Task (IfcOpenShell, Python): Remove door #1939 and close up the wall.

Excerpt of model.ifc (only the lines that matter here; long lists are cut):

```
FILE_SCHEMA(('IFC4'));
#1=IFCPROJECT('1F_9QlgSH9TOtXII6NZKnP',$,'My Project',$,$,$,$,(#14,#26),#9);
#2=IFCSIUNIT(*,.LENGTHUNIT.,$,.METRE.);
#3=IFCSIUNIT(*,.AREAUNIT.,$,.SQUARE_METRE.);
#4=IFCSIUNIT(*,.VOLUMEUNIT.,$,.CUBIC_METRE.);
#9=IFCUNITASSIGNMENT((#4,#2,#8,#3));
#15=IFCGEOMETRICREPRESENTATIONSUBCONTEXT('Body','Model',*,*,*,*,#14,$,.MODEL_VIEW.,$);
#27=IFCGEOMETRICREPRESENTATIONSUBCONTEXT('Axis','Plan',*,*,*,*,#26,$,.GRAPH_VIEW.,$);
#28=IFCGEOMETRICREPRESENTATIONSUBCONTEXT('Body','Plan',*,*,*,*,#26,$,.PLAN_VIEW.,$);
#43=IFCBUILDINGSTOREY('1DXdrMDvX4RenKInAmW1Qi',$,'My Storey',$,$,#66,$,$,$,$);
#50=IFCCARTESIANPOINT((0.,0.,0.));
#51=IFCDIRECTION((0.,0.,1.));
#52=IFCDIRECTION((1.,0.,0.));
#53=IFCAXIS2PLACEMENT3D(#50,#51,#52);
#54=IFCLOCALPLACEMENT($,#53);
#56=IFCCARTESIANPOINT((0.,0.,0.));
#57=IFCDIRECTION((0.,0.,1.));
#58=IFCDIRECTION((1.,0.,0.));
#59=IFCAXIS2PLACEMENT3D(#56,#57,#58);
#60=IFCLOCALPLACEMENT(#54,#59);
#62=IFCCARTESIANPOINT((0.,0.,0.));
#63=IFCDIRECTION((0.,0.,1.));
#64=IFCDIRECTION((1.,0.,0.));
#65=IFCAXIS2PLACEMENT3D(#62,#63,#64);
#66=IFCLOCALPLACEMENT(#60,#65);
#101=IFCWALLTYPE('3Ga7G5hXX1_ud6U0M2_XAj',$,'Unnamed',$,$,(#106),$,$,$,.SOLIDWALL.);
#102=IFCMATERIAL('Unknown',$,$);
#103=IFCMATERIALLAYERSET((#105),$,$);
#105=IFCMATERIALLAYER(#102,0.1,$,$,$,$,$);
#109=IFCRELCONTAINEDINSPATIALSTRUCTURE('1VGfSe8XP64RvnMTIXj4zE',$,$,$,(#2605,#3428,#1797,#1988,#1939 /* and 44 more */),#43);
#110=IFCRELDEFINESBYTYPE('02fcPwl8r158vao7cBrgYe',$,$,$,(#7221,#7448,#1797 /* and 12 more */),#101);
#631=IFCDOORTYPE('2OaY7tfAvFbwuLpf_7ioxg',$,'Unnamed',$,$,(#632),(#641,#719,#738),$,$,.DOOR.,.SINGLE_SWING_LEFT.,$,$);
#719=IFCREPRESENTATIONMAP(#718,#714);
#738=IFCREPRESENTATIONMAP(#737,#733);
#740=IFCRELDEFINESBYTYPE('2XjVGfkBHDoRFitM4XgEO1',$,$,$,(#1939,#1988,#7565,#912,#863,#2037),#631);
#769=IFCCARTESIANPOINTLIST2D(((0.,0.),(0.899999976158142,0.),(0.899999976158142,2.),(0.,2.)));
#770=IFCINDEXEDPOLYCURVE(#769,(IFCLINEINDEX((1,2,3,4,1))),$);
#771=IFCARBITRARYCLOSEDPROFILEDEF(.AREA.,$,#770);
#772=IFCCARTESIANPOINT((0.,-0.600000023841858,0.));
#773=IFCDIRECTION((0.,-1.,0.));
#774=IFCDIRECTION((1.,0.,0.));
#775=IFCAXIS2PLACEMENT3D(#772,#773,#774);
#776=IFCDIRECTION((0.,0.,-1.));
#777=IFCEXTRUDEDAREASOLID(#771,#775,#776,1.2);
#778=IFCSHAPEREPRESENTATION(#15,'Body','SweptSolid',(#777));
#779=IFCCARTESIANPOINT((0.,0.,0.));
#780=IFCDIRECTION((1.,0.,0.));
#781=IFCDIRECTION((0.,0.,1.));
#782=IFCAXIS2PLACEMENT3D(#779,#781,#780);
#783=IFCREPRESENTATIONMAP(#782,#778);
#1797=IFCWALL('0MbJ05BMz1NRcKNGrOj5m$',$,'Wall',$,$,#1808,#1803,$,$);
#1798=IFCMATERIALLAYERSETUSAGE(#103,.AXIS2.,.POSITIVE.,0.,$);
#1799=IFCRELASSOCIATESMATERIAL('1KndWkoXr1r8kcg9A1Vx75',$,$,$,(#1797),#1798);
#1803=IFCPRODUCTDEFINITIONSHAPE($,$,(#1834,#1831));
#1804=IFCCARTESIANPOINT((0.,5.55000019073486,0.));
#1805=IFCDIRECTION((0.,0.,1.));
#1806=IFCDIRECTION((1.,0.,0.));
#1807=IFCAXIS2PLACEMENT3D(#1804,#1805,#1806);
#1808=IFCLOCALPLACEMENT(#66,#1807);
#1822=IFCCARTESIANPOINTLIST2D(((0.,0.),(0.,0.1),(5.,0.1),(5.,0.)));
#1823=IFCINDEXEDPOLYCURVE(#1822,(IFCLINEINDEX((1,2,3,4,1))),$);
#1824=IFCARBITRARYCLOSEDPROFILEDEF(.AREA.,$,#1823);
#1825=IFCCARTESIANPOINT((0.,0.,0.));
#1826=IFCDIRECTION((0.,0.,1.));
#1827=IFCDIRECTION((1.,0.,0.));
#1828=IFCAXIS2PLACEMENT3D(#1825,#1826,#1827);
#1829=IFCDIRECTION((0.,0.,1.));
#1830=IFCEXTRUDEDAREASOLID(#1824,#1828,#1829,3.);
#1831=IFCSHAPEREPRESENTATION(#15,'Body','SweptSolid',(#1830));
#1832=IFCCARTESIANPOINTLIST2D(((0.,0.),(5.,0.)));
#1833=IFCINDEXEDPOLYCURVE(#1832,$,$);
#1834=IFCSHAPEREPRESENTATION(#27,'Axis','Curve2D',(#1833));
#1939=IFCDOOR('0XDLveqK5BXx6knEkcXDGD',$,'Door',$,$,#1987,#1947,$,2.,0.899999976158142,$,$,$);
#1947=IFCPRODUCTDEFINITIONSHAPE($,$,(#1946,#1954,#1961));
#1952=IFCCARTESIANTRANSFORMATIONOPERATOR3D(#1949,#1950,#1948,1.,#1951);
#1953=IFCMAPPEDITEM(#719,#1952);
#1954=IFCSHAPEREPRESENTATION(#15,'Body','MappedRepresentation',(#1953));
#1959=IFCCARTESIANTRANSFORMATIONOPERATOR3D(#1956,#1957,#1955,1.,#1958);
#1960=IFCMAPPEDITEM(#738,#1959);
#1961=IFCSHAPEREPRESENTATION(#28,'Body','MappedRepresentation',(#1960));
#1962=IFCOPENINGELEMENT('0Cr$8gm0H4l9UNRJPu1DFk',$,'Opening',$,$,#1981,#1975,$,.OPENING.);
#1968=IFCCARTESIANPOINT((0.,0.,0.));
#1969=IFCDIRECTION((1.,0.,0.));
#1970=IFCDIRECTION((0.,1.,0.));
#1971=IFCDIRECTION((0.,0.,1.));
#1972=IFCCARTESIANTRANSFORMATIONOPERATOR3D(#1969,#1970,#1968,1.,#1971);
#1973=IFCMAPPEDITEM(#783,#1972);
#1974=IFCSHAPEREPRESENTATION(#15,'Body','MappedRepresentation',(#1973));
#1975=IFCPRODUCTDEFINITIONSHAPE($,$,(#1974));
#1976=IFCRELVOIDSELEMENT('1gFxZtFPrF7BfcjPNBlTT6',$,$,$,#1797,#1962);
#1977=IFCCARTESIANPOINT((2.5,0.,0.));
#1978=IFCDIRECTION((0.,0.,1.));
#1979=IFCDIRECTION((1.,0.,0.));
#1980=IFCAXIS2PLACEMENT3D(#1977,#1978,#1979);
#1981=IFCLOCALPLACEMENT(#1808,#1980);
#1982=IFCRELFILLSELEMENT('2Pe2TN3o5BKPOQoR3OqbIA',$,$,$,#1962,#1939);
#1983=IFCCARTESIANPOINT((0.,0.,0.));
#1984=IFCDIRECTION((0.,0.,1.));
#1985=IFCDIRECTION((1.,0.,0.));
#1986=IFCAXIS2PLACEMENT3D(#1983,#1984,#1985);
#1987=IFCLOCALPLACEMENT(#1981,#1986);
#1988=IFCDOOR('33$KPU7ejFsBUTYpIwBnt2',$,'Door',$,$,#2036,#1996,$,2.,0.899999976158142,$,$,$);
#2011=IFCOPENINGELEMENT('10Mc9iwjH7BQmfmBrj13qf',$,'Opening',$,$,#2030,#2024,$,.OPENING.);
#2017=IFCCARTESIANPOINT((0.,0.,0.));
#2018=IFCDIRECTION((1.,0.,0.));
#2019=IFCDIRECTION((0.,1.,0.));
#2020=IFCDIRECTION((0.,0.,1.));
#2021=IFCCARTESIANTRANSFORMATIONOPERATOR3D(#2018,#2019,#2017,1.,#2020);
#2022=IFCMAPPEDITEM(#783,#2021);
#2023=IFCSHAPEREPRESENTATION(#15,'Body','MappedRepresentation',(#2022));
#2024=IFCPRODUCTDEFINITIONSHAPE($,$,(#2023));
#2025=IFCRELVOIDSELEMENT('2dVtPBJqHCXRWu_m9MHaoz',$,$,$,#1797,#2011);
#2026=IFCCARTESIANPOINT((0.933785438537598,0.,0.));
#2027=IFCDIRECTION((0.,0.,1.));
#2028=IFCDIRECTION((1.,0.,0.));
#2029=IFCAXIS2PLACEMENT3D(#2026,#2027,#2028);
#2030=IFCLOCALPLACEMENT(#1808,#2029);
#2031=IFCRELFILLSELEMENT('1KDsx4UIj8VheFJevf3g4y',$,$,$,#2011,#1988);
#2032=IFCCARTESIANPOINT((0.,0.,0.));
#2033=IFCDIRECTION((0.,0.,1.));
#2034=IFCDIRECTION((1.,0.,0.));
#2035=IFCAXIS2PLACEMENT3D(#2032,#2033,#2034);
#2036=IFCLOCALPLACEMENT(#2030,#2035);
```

```python
import ifcopenshell
import ifcopenshell.api.feature
import ifcopenshell.api.root
import ifcopenshell.geom
import ifcopenshell.util.shape

model = ifcopenshell.open("model.ifc")
settings = ifcopenshell.geom.settings()


def volume(element):
    """Net volume in cubic metres, openings subtracted."""
    shape = ifcopenshell.geom.create_shape(settings, element)
    return ifcopenshell.util.shape.get_volume(shape.geometry)


door = model.by_guid("0XDLveqK5BXx6knEkcXDGD")
opening = door.FillsVoids[0].RelatingOpeningElement
wall = opening.VoidsElements[0].RelatingBuildingElement
before = volume(wall)

ifcopenshell.api.root.remove_product(model, product=door)
ifcopenshell.api.feature.remove_feature(model, feature=opening)

after = volume(wall)

print(f"wall volume {before:.3f} -> {after:.3f} m3")

model.write("model_updated.ifc")
```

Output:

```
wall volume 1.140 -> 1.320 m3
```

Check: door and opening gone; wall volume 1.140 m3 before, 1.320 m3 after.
